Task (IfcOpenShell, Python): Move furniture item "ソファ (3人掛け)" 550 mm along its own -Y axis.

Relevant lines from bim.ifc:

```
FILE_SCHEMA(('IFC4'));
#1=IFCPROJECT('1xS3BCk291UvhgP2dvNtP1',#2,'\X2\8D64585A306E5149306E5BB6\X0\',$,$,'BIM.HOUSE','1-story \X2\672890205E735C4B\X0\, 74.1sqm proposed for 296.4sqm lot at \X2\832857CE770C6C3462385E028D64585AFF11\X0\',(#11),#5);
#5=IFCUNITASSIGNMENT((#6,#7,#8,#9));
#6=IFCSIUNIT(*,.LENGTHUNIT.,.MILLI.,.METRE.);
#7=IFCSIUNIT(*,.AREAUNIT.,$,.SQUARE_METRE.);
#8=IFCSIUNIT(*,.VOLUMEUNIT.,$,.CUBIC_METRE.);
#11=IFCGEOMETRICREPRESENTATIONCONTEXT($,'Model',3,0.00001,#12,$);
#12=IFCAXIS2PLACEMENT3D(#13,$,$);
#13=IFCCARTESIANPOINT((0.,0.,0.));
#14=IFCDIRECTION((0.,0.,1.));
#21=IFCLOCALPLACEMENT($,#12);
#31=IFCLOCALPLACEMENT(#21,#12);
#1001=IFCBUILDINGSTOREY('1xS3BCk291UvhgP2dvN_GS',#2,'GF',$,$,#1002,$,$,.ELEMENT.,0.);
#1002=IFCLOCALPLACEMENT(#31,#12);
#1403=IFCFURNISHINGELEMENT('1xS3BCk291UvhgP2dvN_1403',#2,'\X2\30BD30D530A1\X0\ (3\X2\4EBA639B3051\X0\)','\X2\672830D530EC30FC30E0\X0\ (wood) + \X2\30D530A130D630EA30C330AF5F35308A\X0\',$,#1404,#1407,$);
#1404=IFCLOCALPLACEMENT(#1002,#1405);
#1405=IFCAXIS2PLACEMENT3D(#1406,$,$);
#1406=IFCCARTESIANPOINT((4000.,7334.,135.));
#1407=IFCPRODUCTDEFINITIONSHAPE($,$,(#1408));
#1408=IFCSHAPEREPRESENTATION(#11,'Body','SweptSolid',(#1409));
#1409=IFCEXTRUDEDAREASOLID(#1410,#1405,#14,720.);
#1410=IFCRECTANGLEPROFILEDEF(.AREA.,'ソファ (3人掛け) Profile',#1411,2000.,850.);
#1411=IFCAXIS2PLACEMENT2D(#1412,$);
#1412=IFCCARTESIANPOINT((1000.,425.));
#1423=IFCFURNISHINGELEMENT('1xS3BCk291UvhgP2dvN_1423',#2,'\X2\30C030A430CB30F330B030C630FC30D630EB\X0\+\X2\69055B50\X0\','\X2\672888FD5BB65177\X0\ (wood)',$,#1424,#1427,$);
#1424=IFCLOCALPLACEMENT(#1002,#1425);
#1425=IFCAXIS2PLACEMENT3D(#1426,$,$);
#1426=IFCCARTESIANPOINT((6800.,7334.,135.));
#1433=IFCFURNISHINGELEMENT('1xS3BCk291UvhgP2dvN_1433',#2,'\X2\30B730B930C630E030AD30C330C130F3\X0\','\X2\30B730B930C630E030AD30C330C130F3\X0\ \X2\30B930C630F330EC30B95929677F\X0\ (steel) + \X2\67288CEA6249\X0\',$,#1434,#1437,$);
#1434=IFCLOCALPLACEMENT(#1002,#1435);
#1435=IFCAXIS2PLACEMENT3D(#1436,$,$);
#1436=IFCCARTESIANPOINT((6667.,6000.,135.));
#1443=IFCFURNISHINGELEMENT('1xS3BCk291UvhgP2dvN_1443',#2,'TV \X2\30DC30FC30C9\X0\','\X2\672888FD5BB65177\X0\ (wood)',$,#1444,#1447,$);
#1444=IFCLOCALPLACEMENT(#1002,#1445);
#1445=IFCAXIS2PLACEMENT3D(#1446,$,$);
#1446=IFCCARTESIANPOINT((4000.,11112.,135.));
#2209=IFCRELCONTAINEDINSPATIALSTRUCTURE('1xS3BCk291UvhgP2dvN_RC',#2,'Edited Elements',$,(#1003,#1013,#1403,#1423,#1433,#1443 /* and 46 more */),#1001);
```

```python
import ifcopenshell
import ifcopenshell.api.geometry
import ifcopenshell.util.placement

model = ifcopenshell.open("bim.ifc")

item = model.by_id(1403)
matrix = ifcopenshell.util.placement.get_local_placement(item.ObjectPlacement)
matrix[:3, 3] -= matrix[:3, 1] * 550.0
ifcopenshell.api.geometry.edit_object_placement(model, product=item, matrix=matrix, is_si=False)

print(ifcopenshell.util.placement.get_local_placement(item.ObjectPlacement).round(3) + 0.0)

model.write("bim_edited.ifc")
```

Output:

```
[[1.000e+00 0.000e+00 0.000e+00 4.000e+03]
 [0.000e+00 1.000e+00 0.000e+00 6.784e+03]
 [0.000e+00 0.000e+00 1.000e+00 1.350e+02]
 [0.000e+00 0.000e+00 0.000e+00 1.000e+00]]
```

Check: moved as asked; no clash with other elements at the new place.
